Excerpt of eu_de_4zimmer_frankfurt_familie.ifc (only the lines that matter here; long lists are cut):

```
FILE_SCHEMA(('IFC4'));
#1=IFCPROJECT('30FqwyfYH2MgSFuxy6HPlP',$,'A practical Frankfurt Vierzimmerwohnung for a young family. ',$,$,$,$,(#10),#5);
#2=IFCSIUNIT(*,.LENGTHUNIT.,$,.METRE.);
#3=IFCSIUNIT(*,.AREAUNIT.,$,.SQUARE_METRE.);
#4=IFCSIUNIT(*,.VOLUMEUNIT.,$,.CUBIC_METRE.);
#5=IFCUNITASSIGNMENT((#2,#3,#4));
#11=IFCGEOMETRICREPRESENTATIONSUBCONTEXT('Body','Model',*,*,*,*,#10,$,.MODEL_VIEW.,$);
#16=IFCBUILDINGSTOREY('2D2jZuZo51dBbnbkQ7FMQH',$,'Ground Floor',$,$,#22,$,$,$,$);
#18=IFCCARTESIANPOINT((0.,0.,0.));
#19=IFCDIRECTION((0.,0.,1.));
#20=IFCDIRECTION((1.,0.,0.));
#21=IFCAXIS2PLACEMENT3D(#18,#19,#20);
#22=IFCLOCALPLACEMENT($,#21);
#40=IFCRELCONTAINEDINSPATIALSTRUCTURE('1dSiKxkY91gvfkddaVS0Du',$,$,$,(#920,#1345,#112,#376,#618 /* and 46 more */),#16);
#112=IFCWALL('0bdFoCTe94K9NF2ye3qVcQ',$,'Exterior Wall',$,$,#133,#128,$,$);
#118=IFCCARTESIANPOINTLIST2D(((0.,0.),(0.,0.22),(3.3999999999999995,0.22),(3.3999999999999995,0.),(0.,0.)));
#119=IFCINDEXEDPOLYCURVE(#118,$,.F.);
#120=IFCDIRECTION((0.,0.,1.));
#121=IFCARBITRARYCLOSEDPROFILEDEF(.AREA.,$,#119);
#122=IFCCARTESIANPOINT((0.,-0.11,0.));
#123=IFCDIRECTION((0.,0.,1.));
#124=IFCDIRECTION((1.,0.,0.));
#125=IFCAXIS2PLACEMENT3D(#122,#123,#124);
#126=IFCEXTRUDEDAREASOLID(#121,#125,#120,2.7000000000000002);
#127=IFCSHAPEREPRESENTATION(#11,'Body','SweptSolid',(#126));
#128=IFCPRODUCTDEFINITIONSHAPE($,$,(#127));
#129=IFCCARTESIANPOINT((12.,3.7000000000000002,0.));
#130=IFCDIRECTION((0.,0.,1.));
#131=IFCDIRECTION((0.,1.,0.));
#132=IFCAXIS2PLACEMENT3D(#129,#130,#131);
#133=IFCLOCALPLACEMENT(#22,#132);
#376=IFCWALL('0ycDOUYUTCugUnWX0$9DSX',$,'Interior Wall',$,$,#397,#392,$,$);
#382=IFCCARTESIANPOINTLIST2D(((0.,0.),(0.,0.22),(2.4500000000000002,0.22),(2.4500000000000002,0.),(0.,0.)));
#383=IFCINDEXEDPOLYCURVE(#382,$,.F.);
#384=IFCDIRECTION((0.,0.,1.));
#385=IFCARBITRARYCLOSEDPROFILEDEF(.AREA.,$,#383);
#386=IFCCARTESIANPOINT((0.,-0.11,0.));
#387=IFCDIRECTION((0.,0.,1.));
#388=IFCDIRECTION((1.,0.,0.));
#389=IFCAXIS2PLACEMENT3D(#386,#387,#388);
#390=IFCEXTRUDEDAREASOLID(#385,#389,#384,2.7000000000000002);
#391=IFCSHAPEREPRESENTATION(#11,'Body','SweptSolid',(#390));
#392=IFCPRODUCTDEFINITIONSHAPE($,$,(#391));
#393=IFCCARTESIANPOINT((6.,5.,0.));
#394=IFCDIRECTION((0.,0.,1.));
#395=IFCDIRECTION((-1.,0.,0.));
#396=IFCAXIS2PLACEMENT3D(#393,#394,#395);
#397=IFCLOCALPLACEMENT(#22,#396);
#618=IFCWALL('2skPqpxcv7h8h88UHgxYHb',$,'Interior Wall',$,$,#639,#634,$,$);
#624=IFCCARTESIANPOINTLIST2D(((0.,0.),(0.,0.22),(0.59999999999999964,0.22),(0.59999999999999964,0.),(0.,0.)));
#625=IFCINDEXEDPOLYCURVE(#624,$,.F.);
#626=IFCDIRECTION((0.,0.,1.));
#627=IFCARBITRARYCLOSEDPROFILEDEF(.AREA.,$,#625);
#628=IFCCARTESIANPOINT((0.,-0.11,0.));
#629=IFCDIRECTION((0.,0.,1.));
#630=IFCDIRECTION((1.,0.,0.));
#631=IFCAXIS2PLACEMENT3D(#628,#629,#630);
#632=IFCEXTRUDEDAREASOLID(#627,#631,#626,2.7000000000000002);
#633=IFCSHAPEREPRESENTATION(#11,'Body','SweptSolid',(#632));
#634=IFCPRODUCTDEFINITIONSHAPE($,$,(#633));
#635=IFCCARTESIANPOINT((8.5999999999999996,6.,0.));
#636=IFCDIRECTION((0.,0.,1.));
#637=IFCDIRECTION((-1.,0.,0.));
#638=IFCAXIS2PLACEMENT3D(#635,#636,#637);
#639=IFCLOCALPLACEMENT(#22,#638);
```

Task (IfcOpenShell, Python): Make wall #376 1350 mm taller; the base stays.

```python
import ifcopenshell
import ifcopenshell.geom
import ifcopenshell.util.representation
import ifcopenshell.util.shape

model = ifcopenshell.open("eu_de_4zimmer_frankfurt_familie.ifc")
settings = ifcopenshell.geom.settings()


def volume(element):
    """Net volume in cubic metres, openings subtracted."""
    shape = ifcopenshell.geom.create_shape(settings, element)
    return ifcopenshell.util.shape.get_volume(shape.geometry)


wall = model.by_guid("0ycDOUYUTCugUnWX0$9DSX")
before = volume(wall)

body = ifcopenshell.util.representation.get_representation(wall, "Model", "Body")
solid = body.Items[0]
old_height = solid.Depth
solid.Depth += 1.35
after = volume(wall)

print(f"height {old_height:g} -> {solid.Depth:g}, volume {before:.3f} -> {after:.3f} m3")

model.write("eu_de_4zimmer_frankfurt_familie_updated.ifc")
```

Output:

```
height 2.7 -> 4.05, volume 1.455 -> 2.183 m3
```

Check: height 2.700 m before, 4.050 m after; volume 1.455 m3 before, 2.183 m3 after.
